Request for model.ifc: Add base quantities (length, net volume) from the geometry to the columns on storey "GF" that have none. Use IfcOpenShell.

First a look at what the model holds.

```python
import ifcopenshell
import ifcopenshell.util.element
import ifcopenshell.util.unit

model = ifcopenshell.open("model.ifc")
print(model.schema)
for unit_type in ("LENGTHUNIT", "AREAUNIT", "VOLUMEUNIT"):
    print(unit_type, ifcopenshell.util.unit.calculate_unit_scale(model, unit_type))
storey = next(s for s in model.by_type("IfcBuildingStorey") if s.Name == "GF")
columns = [e for e in ifcopenshell.util.element.get_decomposition(storey) if e.is_a("IfcColumn")]
for e in sorted(columns, key=lambda e: e.id()):
    print(e.id(), e.is_a(), e.Name, list(ifcopenshell.util.element.get_psets(e, qtos_only=True)), sep=" | ")
```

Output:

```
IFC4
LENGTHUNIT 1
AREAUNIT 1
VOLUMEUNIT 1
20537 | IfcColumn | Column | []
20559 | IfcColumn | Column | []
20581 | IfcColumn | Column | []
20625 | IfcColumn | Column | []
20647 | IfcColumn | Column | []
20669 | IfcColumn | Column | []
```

```python
import ifcopenshell
import ifcopenshell.api.pset
import ifcopenshell.geom
import ifcopenshell.util.element
import ifcopenshell.util.shape
import ifcopenshell.util.unit

model = ifcopenshell.open("model.ifc")
unit_scale = ifcopenshell.util.unit.calculate_unit_scale(model)
volume_scale = ifcopenshell.util.unit.calculate_unit_scale(model, "VOLUMEUNIT")
settings = ifcopenshell.geom.settings()

storey = next(s for s in model.by_type("IfcBuildingStorey") if s.Name == "GF")
columns = [e for e in ifcopenshell.util.element.get_decomposition(storey) if e.is_a("IfcColumn")]

for e in sorted(columns, key=lambda e: e.id()):
    if ifcopenshell.util.element.get_psets(e, qtos_only=True, should_inherit=False):
        continue
    # Geometry comes back in metres, in the element's own axes.
    shape = ifcopenshell.geom.create_shape(settings, e)
    values = {
        "Length": ifcopenshell.util.shape.get_z(shape.geometry) / unit_scale,
        "NetVolume": ifcopenshell.util.shape.get_volume(shape.geometry) / volume_scale,
    }
    qto = ifcopenshell.api.pset.add_qto(model, product=e, name="Qto_ColumnBaseQuantities")
    ifcopenshell.api.pset.edit_qto(model, qto=qto, properties=values)
    print(e.id(), {k: round(v, 3) for k, v in values.items()})

model.write("model_v2.ifc")
```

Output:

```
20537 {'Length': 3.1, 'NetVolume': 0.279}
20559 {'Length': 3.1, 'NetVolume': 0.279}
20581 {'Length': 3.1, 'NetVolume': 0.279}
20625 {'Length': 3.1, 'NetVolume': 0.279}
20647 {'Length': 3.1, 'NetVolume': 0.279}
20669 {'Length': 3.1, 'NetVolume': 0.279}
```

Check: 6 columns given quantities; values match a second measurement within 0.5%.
